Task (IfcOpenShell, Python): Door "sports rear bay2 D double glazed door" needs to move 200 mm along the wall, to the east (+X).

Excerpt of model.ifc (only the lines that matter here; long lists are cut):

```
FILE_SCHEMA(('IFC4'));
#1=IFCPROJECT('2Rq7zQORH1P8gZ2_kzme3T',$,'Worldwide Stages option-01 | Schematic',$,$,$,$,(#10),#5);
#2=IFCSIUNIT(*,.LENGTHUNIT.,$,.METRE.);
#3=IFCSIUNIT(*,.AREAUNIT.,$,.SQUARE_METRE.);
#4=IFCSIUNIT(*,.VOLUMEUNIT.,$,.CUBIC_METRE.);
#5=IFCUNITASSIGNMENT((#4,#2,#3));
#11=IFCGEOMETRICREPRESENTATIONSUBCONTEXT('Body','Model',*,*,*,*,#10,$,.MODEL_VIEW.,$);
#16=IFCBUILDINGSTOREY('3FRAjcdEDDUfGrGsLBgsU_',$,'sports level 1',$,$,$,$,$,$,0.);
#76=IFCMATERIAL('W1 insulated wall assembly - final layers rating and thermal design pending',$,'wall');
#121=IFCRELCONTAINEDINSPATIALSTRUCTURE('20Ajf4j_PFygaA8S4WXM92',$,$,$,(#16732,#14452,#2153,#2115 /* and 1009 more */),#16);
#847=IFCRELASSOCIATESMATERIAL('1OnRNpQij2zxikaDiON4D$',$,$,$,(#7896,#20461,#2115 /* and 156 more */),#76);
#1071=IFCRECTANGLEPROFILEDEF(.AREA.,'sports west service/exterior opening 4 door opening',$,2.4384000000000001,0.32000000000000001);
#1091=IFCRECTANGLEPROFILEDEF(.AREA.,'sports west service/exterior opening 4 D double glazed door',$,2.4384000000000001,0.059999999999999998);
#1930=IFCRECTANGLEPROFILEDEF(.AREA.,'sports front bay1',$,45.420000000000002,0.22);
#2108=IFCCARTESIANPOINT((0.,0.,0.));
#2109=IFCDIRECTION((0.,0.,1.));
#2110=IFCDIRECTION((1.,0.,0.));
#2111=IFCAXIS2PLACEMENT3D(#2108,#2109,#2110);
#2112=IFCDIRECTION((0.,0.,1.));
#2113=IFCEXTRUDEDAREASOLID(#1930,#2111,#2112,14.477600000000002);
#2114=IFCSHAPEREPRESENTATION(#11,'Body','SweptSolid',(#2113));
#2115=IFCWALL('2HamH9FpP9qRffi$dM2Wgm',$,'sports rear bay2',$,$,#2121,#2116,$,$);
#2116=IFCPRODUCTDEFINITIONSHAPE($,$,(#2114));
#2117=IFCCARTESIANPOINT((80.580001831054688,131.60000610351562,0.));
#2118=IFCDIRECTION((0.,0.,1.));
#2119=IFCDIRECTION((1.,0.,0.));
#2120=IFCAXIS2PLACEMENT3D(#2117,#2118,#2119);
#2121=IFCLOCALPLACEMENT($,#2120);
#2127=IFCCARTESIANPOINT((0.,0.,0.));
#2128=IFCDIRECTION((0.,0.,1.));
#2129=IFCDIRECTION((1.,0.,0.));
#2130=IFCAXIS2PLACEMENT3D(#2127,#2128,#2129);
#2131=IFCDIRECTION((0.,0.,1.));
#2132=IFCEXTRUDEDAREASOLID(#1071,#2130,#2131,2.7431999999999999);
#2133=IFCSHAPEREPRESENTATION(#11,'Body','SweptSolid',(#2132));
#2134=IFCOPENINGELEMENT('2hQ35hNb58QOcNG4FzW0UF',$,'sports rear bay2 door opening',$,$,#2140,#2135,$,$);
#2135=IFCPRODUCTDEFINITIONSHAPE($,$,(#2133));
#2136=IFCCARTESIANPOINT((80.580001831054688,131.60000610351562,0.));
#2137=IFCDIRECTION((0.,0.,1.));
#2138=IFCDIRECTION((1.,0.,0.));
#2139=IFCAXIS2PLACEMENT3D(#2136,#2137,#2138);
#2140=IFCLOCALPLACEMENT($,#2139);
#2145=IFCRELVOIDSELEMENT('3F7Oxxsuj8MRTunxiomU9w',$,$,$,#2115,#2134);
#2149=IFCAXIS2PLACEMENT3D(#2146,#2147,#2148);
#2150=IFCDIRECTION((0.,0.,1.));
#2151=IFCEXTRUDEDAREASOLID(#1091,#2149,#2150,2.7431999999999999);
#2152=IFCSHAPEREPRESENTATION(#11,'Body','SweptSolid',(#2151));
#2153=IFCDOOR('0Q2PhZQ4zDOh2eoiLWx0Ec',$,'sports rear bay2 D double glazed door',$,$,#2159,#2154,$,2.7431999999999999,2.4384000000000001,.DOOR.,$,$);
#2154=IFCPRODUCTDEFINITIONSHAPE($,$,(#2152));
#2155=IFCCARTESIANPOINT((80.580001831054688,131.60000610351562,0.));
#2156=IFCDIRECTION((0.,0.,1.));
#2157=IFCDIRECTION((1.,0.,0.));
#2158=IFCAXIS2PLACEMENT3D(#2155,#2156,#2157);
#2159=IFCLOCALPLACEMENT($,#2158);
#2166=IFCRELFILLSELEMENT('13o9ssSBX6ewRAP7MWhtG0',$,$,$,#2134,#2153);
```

```python
import ifcopenshell
import ifcopenshell.api.geometry
import ifcopenshell.util.placement
import ifcopenshell.util.unit

model = ifcopenshell.open("model.ifc")
unit_scale = ifcopenshell.util.unit.calculate_unit_scale(model)

door = model.by_id(2153)
opening = door.FillsVoids[0].RelatingOpeningElement
wall = opening.VoidsElements[0].RelatingBuildingElement

wall_matrix = ifcopenshell.util.placement.get_local_placement(wall.ObjectPlacement)
shift = wall_matrix[:3, 0] * 0.2 / unit_scale
before = ifcopenshell.util.placement.get_local_placement(door.ObjectPlacement)[:3, 3].copy()

# The door is not placed relative to its opening, so move both.
for product in (opening, door):
    matrix = ifcopenshell.util.placement.get_local_placement(product.ObjectPlacement)
    matrix[:3, 3] += shift
    ifcopenshell.api.geometry.edit_object_placement(model, product=product, matrix=matrix, is_si=False)

after = ifcopenshell.util.placement.get_local_placement(door.ObjectPlacement)[:3, 3]
print("door moved by", (after - before).round(3) + 0.0)

model.write("model_edited.ifc")
```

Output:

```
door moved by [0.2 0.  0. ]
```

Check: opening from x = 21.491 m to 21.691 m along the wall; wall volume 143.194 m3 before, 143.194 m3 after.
